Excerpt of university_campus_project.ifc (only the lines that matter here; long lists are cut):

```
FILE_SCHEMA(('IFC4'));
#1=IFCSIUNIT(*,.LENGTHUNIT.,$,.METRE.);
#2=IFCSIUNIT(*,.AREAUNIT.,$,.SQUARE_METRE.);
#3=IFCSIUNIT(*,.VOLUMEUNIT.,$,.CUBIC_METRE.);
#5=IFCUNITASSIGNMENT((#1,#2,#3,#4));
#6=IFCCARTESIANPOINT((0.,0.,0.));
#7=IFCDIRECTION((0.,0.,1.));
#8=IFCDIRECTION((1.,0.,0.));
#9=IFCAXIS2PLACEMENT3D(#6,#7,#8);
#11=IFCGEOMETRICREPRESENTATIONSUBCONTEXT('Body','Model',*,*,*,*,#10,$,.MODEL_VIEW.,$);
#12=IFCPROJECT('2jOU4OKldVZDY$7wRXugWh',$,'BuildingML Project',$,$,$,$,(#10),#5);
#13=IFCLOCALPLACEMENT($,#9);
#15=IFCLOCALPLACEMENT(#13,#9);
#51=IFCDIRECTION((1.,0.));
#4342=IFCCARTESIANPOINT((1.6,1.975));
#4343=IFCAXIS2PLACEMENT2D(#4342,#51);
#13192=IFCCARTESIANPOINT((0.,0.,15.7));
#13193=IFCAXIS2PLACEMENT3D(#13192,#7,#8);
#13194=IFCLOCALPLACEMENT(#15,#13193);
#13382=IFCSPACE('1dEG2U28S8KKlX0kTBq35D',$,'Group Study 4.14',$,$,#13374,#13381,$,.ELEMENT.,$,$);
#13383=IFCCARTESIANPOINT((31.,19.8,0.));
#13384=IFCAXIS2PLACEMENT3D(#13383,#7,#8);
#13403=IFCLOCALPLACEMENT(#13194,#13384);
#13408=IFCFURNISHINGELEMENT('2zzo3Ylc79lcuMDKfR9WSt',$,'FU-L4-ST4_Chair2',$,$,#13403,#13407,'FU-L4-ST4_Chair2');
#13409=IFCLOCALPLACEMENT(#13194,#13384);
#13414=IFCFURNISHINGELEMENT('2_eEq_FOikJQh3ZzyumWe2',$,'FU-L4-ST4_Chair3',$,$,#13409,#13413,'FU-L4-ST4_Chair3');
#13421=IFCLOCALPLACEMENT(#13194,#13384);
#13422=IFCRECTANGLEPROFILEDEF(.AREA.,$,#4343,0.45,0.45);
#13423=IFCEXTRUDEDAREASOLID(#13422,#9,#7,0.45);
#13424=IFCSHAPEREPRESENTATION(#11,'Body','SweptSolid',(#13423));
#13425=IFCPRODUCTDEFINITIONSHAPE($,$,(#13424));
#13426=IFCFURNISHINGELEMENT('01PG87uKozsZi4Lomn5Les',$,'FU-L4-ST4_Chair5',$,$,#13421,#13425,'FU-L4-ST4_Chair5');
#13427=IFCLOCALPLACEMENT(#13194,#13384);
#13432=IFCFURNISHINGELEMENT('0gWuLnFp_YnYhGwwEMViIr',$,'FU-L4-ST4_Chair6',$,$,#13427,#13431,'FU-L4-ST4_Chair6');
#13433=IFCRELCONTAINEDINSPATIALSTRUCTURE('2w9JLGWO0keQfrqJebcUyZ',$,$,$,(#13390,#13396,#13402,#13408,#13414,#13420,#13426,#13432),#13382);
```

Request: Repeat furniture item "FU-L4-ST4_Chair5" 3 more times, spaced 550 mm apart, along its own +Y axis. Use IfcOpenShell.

```python
import ifcopenshell
import ifcopenshell.api.geometry
import ifcopenshell.api.root
import ifcopenshell.util.element
import ifcopenshell.util.placement

model = ifcopenshell.open("university_campus_project.ifc")

source = model.by_guid("01PG87uKozsZi4Lomn5Les")
base = ifcopenshell.util.placement.get_local_placement(source.ObjectPlacement)
step = base[:3, 1] * 0.55

for i in range(1, 4):
    copy = ifcopenshell.api.root.copy_class(model, product=source)
    copy.Representation = ifcopenshell.util.element.copy_deep(
        model, source.Representation, exclude=["IfcGeometricRepresentationContext", "IfcRepresentationMap"]
    )
    copy.Tag = None
    matrix = base.copy()
    matrix[:3, 3] += i * step
    print("added at", matrix[:3, 3].round(3) + 0.0)
    ifcopenshell.api.geometry.edit_object_placement(model, product=copy, matrix=matrix, is_si=False)

model.write("university_campus_project-out.ifc")
```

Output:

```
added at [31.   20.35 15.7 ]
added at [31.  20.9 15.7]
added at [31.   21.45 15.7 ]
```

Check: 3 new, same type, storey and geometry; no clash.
